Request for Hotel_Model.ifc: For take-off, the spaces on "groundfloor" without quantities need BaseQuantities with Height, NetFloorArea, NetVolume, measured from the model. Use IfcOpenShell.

First a look at what the model holds.

```python
import ifcopenshell
import ifcopenshell.util.element
import ifcopenshell.util.unit

model = ifcopenshell.open("Hotel_Model.ifc")
print(model.schema)
for unit_type in ("LENGTHUNIT", "AREAUNIT", "VOLUMEUNIT"):
    print(unit_type, ifcopenshell.util.unit.calculate_unit_scale(model, unit_type))
storey = next(s for s in model.by_type("IfcBuildingStorey") if s.Name == "groundfloor")
spaces = [e for e in ifcopenshell.util.element.get_decomposition(storey) if e.is_a("IfcSpace")]
for e in sorted(spaces, key=lambda e: e.id()):
    print(e.id(), e.is_a(), e.Name, list(ifcopenshell.util.element.get_psets(e, qtos_only=True)), sep=" | ")
```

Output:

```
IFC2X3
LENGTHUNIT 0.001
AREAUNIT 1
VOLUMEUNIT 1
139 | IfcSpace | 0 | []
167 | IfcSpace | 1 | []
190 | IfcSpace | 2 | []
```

```python
import ifcopenshell
import ifcopenshell.api.pset
import ifcopenshell.geom
import ifcopenshell.util.element
import ifcopenshell.util.shape
import ifcopenshell.util.unit

model = ifcopenshell.open("Hotel_Model.ifc")
unit_scale = ifcopenshell.util.unit.calculate_unit_scale(model)
area_scale = ifcopenshell.util.unit.calculate_unit_scale(model, "AREAUNIT")
volume_scale = ifcopenshell.util.unit.calculate_unit_scale(model, "VOLUMEUNIT")
settings = ifcopenshell.geom.settings()

storey = next(s for s in model.by_type("IfcBuildingStorey") if s.Name == "groundfloor")
spaces = [e for e in ifcopenshell.util.element.get_decomposition(storey) if e.is_a("IfcSpace")]

for e in sorted(spaces, key=lambda e: e.id()):
    if ifcopenshell.util.element.get_psets(e, qtos_only=True, should_inherit=False):
        continue
    # Geometry comes back in metres, in the element's own axes.
    shape = ifcopenshell.geom.create_shape(settings, e)
    values = {
        "Height": ifcopenshell.util.shape.get_z(shape.geometry) / unit_scale,
        "NetFloorArea": ifcopenshell.util.shape.get_footprint_area(shape.geometry) / area_scale,
        "NetVolume": ifcopenshell.util.shape.get_volume(shape.geometry) / volume_scale,
    }
    qto = ifcopenshell.api.pset.add_qto(model, product=e, name="BaseQuantities")
    ifcopenshell.api.pset.edit_qto(model, qto=qto, properties=values)
    print(e.id(), {k: round(v, 3) for k, v in values.items()})

model.write("Hotel_Model_v2.ifc")
```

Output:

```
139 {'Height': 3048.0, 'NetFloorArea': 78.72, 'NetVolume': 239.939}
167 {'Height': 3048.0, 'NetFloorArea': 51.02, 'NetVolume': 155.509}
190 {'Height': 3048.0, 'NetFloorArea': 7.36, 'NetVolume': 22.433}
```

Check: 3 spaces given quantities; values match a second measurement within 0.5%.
